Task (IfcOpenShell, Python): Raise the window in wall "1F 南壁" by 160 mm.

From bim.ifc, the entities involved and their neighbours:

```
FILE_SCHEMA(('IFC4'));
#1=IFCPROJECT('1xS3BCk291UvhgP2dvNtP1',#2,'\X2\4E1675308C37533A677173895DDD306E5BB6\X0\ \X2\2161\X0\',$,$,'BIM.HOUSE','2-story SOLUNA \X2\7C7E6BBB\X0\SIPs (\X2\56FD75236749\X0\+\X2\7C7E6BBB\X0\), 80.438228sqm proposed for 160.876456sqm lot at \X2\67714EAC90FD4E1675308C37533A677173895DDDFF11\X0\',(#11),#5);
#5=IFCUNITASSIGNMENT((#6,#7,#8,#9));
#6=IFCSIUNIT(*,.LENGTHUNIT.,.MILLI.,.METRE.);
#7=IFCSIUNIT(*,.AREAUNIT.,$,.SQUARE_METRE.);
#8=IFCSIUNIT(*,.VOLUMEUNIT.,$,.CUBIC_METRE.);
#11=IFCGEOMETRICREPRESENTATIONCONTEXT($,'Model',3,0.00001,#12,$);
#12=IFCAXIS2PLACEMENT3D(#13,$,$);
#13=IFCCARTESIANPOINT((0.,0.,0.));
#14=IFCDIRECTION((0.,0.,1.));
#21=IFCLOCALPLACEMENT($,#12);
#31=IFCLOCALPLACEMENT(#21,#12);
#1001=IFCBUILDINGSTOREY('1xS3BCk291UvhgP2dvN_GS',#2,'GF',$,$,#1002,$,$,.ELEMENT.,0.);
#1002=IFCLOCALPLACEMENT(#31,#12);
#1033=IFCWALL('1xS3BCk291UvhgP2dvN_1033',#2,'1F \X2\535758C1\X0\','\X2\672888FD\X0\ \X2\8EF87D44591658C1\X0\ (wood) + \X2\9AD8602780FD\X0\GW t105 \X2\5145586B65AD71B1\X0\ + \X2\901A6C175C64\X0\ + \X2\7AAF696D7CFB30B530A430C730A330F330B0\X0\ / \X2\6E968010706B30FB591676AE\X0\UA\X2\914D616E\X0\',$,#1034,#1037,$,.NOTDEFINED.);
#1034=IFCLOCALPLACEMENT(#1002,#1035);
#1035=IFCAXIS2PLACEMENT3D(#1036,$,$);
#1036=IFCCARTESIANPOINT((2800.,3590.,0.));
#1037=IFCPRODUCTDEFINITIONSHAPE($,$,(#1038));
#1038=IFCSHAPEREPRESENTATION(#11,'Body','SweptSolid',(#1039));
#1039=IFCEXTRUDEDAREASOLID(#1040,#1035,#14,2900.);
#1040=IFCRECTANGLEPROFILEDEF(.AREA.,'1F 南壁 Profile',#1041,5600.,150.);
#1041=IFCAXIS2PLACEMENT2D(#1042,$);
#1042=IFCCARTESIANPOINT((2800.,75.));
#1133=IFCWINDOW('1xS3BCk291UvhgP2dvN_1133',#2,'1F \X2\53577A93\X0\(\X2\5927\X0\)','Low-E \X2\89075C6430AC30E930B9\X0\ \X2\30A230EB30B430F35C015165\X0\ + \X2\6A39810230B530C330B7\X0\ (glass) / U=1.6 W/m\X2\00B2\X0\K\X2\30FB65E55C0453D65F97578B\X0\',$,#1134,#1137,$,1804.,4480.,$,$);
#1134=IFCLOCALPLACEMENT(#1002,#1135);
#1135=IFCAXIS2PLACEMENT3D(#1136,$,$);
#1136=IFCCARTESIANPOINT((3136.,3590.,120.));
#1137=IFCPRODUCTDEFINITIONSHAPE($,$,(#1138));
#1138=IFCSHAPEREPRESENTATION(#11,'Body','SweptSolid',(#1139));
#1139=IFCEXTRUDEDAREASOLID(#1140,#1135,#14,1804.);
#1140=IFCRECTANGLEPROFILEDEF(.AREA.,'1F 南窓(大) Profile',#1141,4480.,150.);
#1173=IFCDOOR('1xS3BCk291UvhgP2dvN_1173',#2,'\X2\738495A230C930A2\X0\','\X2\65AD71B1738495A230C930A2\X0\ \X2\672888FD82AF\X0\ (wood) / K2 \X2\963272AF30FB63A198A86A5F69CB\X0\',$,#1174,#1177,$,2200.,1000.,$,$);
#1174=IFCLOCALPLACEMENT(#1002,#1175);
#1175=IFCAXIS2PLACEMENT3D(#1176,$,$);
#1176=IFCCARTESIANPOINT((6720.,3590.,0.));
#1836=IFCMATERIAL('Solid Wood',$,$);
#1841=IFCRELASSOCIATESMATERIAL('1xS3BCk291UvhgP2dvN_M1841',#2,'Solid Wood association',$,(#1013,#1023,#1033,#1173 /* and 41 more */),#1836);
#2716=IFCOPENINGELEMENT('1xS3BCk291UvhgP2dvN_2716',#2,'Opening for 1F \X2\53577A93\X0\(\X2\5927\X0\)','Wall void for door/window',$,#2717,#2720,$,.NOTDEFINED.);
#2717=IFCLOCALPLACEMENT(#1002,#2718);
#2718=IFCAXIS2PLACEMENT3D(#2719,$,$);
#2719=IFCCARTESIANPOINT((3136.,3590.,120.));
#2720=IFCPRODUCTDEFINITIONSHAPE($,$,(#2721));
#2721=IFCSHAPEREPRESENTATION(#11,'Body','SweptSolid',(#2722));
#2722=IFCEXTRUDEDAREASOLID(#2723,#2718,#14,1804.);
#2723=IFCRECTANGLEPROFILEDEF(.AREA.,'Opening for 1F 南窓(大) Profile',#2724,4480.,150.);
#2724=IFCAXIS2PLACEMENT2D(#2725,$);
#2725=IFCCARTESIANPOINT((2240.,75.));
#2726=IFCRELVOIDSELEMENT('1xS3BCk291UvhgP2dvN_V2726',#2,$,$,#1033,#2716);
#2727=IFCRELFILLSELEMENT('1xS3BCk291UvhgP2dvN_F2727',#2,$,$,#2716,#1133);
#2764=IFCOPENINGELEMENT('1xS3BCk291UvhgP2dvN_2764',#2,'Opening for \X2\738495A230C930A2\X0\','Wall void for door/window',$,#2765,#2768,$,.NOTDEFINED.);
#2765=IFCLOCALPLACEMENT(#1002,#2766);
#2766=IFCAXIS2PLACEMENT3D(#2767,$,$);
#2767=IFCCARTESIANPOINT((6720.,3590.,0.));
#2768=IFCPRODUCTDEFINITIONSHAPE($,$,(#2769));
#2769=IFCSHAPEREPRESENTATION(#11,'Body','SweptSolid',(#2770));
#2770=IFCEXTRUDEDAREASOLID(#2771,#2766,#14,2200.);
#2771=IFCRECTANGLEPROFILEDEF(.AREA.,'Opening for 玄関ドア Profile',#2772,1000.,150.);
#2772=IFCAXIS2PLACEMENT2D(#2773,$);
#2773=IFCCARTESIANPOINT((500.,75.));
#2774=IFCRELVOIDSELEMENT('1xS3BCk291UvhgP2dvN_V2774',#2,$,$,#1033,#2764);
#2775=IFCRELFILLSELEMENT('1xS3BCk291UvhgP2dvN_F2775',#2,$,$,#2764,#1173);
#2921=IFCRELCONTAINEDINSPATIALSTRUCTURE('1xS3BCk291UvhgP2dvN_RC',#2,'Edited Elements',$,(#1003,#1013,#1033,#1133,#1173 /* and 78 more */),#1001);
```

```python
import numpy as np
import ifcopenshell
import ifcopenshell.api.geometry
import ifcopenshell.util.placement
import ifcopenshell.util.unit

model = ifcopenshell.open("bim.ifc")
unit_scale = ifcopenshell.util.unit.calculate_unit_scale(model)

window = model.by_guid("1xS3BCk291UvhgP2dvN_1133")
opening = window.FillsVoids[0].RelatingOpeningElement
dz = 160.0

shift = np.array([0.0, 0.0, dz])
# The window is not placed relative to its opening, so move both.
for product in (opening, window):
    matrix = ifcopenshell.util.placement.get_local_placement(product.ObjectPlacement)
    matrix[:3, 3] += shift
    ifcopenshell.api.geometry.edit_object_placement(model, product=product, matrix=matrix, is_si=False)

print(f"moved by {dz * unit_scale:+.3f} m")

model.write("bim_edited.ifc")
```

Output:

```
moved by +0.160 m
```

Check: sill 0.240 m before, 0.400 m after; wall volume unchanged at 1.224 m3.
